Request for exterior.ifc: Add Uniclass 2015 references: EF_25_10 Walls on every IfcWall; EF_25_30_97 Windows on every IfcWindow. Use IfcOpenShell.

First a look at what the model holds.

```python
import ifcopenshell

model = ifcopenshell.open("exterior.ifc")
print(model.schema)
print("classifications:", [c.Name for c in model.by_type("IfcClassification")])
for ifc_class in ("IfcDoor", "IfcRoof", "IfcStair", "IfcWall", "IfcWindow"):
    print(ifc_class, len(model.by_type(ifc_class)))
```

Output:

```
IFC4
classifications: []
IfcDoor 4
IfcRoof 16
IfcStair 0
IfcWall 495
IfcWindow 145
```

```python
import ifcopenshell
import ifcopenshell.api.classification

model = ifcopenshell.open("exterior.ifc")

system = ifcopenshell.api.classification.add_classification(model, classification="Uniclass 2015")

codes = {
    "IfcWall": ("EF_25_10", "Walls"),
    "IfcWindow": ("EF_25_30_97", "Windows"),
}
for ifc_class, (code, name) in codes.items():
    products = model.by_type(ifc_class)
    ifcopenshell.api.classification.add_reference(
        model, products=products, classification=system, identification=code, name=name
    )
    print(code, len(products))

model.write("exterior-out.ifc")
```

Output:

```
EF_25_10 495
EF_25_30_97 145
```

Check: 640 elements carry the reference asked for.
